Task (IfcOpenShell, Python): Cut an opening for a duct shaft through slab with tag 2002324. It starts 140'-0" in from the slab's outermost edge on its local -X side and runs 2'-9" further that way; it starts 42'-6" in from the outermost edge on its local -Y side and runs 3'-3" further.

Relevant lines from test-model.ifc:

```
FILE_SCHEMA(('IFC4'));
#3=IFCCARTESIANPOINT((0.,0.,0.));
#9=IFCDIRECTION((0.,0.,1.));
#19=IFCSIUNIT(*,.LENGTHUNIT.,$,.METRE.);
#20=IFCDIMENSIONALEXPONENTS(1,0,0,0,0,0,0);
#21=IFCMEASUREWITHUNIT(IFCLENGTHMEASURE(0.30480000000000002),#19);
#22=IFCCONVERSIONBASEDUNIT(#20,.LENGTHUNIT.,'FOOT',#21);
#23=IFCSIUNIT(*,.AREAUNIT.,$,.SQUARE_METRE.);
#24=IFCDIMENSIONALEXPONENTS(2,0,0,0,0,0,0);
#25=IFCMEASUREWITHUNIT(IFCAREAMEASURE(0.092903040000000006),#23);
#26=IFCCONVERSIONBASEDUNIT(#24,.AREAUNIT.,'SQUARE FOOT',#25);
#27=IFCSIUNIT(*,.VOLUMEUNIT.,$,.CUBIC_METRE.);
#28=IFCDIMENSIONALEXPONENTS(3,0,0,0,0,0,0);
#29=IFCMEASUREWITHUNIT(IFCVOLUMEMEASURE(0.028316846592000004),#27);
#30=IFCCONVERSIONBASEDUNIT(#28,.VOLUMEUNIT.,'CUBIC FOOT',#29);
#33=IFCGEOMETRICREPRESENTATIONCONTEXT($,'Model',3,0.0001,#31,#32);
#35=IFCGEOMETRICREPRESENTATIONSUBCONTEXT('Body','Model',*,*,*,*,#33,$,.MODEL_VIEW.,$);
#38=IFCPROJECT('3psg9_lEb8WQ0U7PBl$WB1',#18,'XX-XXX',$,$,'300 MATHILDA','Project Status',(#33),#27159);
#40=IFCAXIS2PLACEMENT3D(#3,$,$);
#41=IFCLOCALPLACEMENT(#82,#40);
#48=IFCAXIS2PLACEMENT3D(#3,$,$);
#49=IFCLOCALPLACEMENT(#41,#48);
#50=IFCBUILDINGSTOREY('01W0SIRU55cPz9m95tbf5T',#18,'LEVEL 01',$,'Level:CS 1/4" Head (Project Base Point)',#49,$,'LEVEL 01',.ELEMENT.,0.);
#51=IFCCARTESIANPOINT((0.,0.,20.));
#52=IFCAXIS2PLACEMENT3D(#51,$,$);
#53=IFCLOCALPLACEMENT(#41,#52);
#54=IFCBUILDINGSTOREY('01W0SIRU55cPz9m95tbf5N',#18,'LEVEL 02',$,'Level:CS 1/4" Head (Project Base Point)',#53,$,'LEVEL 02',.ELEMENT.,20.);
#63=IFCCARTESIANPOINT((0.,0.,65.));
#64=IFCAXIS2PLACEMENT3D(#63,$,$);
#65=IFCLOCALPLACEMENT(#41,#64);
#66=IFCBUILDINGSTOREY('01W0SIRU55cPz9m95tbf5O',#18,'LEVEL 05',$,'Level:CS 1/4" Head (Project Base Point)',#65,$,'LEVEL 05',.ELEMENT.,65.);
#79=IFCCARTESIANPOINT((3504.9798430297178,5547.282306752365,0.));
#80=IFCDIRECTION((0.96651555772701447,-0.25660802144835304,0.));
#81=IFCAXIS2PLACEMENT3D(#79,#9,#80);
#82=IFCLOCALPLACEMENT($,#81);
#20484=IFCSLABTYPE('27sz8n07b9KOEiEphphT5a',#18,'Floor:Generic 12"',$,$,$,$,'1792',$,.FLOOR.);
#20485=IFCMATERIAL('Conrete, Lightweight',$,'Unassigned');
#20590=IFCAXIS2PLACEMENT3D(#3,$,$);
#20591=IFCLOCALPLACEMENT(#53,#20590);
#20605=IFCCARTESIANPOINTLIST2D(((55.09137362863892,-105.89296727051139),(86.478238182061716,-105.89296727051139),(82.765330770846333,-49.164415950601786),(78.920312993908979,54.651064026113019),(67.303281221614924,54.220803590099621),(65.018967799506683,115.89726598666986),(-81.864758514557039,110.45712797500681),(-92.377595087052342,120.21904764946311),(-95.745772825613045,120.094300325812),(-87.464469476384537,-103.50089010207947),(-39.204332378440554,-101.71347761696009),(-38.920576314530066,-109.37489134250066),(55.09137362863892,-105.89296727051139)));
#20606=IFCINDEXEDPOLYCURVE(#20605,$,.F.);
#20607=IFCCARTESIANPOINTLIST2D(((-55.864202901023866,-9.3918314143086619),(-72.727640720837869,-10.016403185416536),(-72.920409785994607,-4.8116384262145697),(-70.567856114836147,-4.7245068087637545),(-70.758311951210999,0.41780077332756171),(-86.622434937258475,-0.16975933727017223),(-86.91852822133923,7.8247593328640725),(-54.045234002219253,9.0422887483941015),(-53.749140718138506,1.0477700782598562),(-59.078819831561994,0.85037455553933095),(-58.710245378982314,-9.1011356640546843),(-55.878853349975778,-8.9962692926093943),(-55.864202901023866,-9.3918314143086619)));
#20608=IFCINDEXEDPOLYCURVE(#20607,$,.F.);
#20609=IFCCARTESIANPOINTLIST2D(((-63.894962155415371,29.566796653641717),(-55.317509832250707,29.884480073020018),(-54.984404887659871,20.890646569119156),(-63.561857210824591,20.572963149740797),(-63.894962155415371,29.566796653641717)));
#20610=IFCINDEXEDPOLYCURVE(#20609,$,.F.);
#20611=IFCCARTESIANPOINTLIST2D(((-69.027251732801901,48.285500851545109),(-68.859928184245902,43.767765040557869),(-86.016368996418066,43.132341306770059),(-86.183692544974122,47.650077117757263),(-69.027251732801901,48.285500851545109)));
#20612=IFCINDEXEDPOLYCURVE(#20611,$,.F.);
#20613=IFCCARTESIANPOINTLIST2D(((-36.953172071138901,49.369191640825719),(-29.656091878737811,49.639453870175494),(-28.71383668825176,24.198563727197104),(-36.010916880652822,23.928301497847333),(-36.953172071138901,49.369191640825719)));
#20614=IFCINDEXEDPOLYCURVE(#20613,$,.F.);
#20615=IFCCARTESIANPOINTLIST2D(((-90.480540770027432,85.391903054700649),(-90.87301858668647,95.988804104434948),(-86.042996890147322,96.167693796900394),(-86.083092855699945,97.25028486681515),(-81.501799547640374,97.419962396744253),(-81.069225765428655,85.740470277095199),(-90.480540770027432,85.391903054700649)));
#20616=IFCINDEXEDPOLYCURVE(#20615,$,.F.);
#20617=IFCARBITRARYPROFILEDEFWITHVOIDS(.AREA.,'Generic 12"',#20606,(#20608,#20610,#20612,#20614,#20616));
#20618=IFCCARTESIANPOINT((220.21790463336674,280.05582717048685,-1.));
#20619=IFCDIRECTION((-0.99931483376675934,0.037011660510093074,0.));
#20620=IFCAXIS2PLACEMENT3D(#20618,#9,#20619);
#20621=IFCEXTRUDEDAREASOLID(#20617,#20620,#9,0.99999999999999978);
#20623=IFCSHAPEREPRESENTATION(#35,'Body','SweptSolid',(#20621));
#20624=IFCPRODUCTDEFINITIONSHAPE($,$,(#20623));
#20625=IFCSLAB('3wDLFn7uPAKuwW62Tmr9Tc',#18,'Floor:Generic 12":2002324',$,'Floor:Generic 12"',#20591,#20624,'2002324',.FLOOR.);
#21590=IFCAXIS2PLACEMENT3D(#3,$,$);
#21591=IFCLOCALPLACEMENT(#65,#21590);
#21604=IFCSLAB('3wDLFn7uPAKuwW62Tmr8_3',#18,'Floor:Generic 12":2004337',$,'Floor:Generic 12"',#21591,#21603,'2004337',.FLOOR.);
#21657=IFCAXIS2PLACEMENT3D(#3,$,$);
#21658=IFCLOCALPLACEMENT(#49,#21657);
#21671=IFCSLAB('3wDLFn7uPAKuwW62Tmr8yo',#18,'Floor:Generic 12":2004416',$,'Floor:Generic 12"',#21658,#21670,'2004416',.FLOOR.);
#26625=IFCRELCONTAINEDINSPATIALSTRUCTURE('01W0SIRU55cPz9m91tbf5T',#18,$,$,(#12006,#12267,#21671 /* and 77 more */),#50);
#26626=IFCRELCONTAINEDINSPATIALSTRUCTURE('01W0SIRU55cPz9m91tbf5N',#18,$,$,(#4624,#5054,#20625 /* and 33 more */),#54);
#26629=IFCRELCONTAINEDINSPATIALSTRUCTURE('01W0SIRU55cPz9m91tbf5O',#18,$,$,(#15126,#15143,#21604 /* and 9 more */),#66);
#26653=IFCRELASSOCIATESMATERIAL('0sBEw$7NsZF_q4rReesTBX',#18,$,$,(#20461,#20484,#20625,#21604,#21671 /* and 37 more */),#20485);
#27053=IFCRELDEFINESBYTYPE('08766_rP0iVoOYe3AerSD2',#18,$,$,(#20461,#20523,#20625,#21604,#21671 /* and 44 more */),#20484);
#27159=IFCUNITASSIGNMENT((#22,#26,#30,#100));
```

```python
import numpy as np
import ifcopenshell
import ifcopenshell.api.feature
import ifcopenshell.api.geometry
import ifcopenshell.api.root
import ifcopenshell.geom
import ifcopenshell.util.placement
import ifcopenshell.util.representation
import ifcopenshell.util.shape
import ifcopenshell.util.unit

model = ifcopenshell.open("test-model.ifc")
unit_scale = ifcopenshell.util.unit.calculate_unit_scale(model)
settings = ifcopenshell.geom.settings()


def volume(element):
    """Net volume in cubic metres, openings subtracted."""
    shape = ifcopenshell.geom.create_shape(settings, element)
    return ifcopenshell.util.shape.get_volume(shape.geometry)


slab = model.by_guid("3wDLFn7uPAKuwW62Tmr9Tc")
before = volume(slab)

# Extent in the slab's own axes, in metres. The edges named are its -X and -Y sides.
slab_shape = ifcopenshell.geom.create_shape(settings, slab)
vertices = ifcopenshell.util.shape.get_vertices(slab_shape.geometry)
x_min, y_min, bottom = vertices.min(axis=0)
top = vertices[:, 2].max()

opening = ifcopenshell.api.root.create_entity(model, ifc_class="IfcOpeningElement", name="Duct shaft opening", predefined_type="OPENING")
context = ifcopenshell.util.representation.get_context(model, "Model", "Body", "MODEL_VIEW")
width, depth = 0.8382, 0.9906
outline = [(0.0, 0.0), (width, 0.0), (width, depth), (0.0, depth), (0.0, 0.0)]
# Overshoot both faces by 50 mm so the cut is clean.
shape = ifcopenshell.api.geometry.add_slab_representation(
    model, context=context, depth=top - bottom + 0.1, polyline=outline
)
ifcopenshell.api.geometry.assign_representation(model, product=opening, representation=shape)

matrix = ifcopenshell.util.placement.get_local_placement(slab.ObjectPlacement)
matrix[:, 3] = matrix @ np.append(np.array([x_min + 42.672, y_min + 12.954, bottom - 0.05]) / unit_scale, 1.0)
ifcopenshell.api.geometry.edit_object_placement(model, product=opening, matrix=matrix, is_si=False)
ifcopenshell.api.feature.add_feature(model, feature=opening, element=slab)

after = volume(slab)

print(f"slab volume {before:.3f} -> {after:.3f} m3")

model.write("test-model_updated.ifc")
```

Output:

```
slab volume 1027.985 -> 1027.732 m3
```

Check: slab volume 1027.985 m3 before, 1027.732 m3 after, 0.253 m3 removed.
